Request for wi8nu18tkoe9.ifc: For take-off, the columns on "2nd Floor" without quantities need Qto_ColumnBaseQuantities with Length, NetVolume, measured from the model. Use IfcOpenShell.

First a look at what the model holds.

```python
import ifcopenshell
import ifcopenshell.util.element
import ifcopenshell.util.unit

model = ifcopenshell.open("wi8nu18tkoe9.ifc")
print(model.schema)
for unit_type in ("LENGTHUNIT", "AREAUNIT", "VOLUMEUNIT"):
    print(unit_type, ifcopenshell.util.unit.calculate_unit_scale(model, unit_type))
storey = next(s for s in model.by_type("IfcBuildingStorey") if s.Name == "2nd Floor")
columns = [e for e in ifcopenshell.util.element.get_decomposition(storey) if e.is_a("IfcColumn")]
for e in sorted(columns, key=lambda e: e.id()):
    print(e.id(), e.is_a(), e.Name, list(ifcopenshell.util.element.get_psets(e, qtos_only=True)), sep=" | ")
```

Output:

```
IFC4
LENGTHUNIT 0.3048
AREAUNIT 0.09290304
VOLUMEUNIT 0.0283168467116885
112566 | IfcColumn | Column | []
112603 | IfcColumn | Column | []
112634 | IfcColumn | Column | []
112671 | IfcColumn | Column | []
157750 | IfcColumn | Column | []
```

```python
import ifcopenshell
import ifcopenshell.api.pset
import ifcopenshell.geom
import ifcopenshell.util.element
import ifcopenshell.util.shape
import ifcopenshell.util.unit

model = ifcopenshell.open("wi8nu18tkoe9.ifc")
unit_scale = ifcopenshell.util.unit.calculate_unit_scale(model)
volume_scale = ifcopenshell.util.unit.calculate_unit_scale(model, "VOLUMEUNIT")
settings = ifcopenshell.geom.settings()

storey = next(s for s in model.by_type("IfcBuildingStorey") if s.Name == "2nd Floor")
columns = [e for e in ifcopenshell.util.element.get_decomposition(storey) if e.is_a("IfcColumn")]

for e in sorted(columns, key=lambda e: e.id()):
    if ifcopenshell.util.element.get_psets(e, qtos_only=True, should_inherit=False):
        continue
    # Geometry comes back in metres, in the element's own axes.
    shape = ifcopenshell.geom.create_shape(settings, e)
    values = {
        "Length": ifcopenshell.util.shape.get_z(shape.geometry) / unit_scale,
        "NetVolume": ifcopenshell.util.shape.get_volume(shape.geometry) / volume_scale,
    }
    qto = ifcopenshell.api.pset.add_qto(model, product=e, name="Qto_ColumnBaseQuantities")
    ifcopenshell.api.pset.edit_qto(model, qto=qto, properties=values)
    print(e.id(), {k: round(v, 3) for k, v in values.items()})

model.write("wi8nu18tkoe9_v2.ifc")
```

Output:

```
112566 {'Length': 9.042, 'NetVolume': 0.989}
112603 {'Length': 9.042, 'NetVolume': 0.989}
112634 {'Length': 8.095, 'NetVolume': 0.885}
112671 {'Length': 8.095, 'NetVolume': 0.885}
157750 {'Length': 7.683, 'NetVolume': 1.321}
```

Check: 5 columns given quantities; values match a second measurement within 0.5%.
